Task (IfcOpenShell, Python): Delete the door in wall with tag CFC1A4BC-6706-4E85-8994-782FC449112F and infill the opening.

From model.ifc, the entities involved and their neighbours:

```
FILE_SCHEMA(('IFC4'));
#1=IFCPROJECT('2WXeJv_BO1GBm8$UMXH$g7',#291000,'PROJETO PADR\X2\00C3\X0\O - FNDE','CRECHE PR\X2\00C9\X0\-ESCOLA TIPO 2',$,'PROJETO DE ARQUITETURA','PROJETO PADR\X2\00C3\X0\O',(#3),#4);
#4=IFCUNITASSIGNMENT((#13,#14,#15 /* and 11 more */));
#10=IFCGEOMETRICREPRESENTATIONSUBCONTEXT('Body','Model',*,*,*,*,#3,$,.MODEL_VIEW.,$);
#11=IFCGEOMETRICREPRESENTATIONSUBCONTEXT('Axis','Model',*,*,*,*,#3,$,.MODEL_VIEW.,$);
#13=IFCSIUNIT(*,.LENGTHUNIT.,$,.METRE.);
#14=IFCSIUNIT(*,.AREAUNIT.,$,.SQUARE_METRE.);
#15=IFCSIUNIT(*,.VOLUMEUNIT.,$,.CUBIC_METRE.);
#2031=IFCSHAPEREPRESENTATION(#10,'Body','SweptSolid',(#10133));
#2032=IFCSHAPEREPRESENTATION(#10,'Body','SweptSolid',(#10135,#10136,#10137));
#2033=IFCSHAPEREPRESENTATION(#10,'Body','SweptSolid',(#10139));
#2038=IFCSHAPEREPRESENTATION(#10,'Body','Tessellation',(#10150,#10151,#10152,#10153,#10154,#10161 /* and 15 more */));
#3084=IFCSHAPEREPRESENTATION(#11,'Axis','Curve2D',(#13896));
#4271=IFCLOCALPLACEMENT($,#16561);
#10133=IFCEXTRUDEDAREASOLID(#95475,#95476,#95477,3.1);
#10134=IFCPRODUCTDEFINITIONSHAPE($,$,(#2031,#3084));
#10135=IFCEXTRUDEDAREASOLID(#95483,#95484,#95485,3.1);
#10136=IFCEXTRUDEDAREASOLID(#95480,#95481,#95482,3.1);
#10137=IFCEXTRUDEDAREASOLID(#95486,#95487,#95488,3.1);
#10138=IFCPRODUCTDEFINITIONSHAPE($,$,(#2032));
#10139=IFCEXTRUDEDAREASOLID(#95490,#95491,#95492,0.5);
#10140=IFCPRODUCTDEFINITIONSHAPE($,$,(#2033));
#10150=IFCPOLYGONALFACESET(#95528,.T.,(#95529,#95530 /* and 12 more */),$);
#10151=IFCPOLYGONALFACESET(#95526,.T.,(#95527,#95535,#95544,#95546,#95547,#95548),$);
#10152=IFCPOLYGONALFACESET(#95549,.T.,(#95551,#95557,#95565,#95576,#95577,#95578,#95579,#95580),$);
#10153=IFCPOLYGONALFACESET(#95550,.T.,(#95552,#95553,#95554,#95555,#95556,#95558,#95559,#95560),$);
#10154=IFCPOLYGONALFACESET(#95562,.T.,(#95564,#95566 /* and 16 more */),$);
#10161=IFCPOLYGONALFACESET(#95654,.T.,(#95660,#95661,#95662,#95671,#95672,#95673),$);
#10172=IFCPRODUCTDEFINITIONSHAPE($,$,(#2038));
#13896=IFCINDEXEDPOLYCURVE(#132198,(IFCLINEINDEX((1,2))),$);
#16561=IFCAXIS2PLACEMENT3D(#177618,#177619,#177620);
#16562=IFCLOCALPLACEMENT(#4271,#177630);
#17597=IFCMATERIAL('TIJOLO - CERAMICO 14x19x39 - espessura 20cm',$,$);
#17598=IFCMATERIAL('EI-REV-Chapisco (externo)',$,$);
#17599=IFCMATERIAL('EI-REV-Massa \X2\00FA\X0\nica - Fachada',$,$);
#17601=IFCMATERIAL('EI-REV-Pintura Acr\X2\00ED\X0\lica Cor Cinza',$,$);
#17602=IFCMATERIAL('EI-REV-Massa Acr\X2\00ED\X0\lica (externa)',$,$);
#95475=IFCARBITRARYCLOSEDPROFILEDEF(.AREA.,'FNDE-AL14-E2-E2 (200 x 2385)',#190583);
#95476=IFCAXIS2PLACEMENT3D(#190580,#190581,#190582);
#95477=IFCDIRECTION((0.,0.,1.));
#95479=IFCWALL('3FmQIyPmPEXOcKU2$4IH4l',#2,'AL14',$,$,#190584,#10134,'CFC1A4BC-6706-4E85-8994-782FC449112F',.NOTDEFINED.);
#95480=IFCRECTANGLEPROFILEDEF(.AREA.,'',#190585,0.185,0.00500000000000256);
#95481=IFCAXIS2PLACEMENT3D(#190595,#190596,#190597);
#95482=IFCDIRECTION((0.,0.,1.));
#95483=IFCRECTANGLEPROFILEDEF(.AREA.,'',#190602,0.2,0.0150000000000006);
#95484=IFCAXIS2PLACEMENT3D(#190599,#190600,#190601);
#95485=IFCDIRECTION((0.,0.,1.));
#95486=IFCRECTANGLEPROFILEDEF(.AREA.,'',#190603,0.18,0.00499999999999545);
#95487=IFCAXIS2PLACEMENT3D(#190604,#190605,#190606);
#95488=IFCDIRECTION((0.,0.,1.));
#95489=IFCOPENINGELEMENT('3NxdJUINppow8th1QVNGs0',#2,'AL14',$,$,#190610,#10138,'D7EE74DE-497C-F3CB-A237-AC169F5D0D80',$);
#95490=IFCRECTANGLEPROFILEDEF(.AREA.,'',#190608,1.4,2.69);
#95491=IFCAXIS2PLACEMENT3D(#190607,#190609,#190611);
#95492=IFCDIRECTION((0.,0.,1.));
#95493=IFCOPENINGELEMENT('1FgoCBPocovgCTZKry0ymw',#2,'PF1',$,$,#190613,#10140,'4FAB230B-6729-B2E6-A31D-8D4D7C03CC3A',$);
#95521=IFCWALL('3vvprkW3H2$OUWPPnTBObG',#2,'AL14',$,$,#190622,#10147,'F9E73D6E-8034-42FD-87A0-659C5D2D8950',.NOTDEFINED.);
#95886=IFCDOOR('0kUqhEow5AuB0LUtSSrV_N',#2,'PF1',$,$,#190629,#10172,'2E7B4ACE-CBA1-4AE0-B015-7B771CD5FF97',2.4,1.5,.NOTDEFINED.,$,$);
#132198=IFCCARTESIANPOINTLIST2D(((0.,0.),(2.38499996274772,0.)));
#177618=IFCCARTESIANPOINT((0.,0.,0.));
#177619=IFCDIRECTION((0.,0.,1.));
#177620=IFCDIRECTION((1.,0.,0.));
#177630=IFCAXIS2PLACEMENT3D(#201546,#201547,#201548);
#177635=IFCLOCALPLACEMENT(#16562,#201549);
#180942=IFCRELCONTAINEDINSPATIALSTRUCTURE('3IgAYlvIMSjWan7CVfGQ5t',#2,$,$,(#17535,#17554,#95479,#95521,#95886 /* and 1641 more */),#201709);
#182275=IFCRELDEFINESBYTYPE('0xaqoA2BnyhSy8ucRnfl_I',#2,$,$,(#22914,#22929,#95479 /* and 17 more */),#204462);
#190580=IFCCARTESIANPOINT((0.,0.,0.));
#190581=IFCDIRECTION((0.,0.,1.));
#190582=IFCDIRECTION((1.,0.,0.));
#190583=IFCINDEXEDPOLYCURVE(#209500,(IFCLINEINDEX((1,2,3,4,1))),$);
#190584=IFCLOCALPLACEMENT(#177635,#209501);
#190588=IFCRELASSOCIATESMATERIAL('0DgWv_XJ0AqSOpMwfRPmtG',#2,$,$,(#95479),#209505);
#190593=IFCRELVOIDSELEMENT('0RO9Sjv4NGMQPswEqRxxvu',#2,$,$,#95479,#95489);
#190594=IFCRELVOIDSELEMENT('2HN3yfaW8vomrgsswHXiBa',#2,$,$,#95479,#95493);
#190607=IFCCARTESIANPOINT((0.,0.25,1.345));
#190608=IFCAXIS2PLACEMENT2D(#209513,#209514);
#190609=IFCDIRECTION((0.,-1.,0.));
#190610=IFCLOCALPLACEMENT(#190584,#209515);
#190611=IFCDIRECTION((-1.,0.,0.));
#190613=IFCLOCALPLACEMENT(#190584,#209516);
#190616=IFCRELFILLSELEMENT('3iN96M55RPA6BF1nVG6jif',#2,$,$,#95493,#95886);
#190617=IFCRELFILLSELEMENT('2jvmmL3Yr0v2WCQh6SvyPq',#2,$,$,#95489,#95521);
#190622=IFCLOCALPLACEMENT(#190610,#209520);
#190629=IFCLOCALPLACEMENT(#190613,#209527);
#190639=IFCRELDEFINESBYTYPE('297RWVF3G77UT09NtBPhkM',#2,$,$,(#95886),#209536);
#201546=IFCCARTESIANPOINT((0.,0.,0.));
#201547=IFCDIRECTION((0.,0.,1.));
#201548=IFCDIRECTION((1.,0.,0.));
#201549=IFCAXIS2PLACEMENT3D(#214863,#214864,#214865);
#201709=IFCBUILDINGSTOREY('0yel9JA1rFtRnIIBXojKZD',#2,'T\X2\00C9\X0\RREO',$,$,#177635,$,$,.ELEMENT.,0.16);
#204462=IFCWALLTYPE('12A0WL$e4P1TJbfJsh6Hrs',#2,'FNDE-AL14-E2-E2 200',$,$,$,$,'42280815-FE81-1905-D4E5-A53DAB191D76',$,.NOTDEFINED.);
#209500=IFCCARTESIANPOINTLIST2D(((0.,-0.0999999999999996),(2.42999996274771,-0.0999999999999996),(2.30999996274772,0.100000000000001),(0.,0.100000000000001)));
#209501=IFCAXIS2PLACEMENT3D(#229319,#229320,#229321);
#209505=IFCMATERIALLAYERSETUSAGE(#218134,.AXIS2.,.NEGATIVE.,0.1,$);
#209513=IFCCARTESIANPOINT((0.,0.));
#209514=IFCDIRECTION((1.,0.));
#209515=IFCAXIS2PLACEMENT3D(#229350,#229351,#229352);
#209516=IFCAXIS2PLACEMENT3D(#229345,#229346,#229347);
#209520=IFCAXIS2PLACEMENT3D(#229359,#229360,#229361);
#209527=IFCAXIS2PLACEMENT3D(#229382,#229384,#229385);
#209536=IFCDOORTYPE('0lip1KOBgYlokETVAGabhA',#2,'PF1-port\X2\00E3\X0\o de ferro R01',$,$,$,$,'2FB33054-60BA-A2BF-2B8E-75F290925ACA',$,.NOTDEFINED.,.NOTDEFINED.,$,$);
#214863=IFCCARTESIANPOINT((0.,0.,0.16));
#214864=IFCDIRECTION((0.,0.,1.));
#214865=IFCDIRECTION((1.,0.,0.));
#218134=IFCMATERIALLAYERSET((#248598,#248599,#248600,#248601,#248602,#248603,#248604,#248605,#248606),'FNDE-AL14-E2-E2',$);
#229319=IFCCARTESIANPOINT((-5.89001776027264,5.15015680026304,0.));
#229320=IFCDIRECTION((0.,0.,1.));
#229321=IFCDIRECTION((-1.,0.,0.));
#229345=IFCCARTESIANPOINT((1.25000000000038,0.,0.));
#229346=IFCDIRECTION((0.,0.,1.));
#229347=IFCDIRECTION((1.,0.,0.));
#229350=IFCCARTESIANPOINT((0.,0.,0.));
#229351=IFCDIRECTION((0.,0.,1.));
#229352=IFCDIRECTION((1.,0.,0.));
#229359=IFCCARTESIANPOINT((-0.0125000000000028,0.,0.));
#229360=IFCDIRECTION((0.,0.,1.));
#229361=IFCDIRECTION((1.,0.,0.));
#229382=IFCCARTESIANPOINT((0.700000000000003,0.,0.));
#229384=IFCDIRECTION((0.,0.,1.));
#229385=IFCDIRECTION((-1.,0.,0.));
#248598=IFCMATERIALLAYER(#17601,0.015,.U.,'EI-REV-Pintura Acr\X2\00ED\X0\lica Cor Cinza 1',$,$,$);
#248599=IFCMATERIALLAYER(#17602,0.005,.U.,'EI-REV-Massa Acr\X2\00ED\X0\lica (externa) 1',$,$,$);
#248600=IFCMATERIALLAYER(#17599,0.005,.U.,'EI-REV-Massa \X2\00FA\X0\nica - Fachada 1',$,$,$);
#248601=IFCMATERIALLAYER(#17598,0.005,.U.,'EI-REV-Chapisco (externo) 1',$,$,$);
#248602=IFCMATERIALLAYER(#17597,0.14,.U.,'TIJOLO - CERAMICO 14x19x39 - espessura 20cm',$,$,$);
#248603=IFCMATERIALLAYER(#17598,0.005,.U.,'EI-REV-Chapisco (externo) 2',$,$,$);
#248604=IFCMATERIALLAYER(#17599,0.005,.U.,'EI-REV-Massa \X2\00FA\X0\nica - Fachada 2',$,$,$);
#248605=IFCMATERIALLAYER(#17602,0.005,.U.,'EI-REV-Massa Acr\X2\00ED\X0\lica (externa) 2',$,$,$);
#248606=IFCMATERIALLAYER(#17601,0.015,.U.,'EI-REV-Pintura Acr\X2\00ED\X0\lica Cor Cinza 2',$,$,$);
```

```python
import ifcopenshell
import ifcopenshell.api.feature
import ifcopenshell.api.root
import ifcopenshell.geom
import ifcopenshell.util.shape

model = ifcopenshell.open("model.ifc")
settings = ifcopenshell.geom.settings()


def volume(element):
    """Net volume in cubic metres, openings subtracted."""
    shape = ifcopenshell.geom.create_shape(settings, element)
    return ifcopenshell.util.shape.get_volume(shape.geometry)


door = model.by_guid("0kUqhEow5AuB0LUtSSrV_N")
opening = door.FillsVoids[0].RelatingOpeningElement
wall = opening.VoidsElements[0].RelatingBuildingElement
before = volume(wall)

ifcopenshell.api.root.remove_product(model, product=door)
ifcopenshell.api.feature.remove_feature(model, feature=opening)

after = volume(wall)

print(f"wall volume {before:.3f} -> {after:.3f} m3")

model.write("model-out.ifc")
```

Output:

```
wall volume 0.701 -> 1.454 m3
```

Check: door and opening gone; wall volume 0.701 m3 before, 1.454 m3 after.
